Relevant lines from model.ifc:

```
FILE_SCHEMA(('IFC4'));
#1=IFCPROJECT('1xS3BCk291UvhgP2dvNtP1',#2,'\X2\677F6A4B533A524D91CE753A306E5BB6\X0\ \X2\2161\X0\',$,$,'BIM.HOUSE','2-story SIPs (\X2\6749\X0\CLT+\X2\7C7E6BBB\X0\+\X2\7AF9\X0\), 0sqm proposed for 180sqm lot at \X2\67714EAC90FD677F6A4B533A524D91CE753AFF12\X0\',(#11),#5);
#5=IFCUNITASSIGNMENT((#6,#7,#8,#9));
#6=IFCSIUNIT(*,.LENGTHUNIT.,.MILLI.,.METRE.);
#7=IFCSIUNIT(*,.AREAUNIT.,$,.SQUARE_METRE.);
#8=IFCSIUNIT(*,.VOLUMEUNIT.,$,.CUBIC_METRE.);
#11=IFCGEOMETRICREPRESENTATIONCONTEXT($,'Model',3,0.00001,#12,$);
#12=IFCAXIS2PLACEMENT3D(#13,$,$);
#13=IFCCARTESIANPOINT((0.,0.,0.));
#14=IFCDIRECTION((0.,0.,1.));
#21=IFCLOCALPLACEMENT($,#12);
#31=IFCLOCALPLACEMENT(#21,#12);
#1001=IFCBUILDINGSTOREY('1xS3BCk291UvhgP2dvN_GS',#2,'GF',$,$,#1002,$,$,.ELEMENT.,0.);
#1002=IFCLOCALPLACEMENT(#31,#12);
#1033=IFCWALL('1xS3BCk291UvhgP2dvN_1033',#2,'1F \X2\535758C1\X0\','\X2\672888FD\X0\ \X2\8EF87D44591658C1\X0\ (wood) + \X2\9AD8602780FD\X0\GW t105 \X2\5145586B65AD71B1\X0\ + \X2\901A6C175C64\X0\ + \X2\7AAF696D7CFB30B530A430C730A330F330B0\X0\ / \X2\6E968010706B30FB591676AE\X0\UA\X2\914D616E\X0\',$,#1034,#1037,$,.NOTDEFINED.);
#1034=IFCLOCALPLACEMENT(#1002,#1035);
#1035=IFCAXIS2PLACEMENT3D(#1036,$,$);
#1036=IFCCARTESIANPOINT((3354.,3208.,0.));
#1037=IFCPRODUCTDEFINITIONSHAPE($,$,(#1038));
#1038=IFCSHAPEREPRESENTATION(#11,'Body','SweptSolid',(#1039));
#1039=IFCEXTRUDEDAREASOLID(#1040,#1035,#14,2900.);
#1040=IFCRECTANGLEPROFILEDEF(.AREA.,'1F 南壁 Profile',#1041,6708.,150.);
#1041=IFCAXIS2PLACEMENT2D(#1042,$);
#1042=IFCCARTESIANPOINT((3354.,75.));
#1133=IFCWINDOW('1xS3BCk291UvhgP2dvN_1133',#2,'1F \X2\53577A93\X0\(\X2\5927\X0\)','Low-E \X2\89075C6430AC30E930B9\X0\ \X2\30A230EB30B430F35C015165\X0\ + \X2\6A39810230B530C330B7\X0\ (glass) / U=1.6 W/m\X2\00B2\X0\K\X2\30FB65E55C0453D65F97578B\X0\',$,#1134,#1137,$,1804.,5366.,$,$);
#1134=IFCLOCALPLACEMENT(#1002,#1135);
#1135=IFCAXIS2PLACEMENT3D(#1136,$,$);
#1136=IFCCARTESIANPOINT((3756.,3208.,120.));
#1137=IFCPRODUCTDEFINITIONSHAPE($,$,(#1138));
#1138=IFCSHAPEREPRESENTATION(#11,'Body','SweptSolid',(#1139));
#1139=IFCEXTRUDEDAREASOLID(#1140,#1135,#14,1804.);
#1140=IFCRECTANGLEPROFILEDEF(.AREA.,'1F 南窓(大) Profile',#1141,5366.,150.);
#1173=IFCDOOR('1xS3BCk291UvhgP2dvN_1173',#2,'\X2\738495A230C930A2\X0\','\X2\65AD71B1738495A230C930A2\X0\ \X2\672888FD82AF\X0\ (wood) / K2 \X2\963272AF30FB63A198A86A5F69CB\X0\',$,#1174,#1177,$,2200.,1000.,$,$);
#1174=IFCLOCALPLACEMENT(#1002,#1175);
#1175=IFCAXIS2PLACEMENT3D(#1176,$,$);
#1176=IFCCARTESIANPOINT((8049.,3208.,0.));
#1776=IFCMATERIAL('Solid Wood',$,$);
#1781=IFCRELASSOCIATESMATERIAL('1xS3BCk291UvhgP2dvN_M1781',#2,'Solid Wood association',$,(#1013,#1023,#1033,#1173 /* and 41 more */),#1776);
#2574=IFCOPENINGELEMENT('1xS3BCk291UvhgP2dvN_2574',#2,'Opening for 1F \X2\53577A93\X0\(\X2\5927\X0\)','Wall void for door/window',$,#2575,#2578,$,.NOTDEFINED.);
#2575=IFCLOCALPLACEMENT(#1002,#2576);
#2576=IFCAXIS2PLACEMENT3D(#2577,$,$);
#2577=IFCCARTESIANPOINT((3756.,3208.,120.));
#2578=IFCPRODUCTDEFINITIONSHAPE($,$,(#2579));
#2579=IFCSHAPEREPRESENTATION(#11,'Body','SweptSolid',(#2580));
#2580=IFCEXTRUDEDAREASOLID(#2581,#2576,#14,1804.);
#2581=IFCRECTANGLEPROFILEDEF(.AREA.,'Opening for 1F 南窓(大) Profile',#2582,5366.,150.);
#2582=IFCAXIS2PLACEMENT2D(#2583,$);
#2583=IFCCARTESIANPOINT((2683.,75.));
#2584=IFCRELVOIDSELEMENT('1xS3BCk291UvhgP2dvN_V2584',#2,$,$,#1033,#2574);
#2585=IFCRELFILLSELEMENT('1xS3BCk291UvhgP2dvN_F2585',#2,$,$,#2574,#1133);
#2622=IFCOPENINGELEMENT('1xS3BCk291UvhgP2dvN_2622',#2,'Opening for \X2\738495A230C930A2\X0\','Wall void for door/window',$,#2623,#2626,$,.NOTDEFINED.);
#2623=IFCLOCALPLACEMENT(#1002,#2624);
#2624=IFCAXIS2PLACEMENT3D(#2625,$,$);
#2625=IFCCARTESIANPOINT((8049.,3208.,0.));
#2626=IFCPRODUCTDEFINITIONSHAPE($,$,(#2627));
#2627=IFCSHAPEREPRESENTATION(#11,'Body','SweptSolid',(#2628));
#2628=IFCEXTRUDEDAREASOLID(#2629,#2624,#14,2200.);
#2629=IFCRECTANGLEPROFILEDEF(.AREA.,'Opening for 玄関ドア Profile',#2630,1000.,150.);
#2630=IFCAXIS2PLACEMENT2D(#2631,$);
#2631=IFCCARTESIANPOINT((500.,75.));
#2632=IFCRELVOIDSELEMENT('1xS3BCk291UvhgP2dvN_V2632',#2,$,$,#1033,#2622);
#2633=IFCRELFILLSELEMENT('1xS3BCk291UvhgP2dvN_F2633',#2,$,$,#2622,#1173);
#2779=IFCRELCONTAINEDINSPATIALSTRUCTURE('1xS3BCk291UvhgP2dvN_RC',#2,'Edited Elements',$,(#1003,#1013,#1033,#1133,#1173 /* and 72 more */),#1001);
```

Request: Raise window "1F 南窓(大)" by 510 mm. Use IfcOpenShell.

```python
import numpy as np
import ifcopenshell
import ifcopenshell.api.geometry
import ifcopenshell.util.placement
import ifcopenshell.util.unit

model = ifcopenshell.open("model.ifc")
unit_scale = ifcopenshell.util.unit.calculate_unit_scale(model)

window = model.by_id(1133)
opening = window.FillsVoids[0].RelatingOpeningElement
dz = 0.51 / unit_scale

shift = np.array([0.0, 0.0, dz])
# The window is not placed relative to its opening, so move both.
for product in (opening, window):
    matrix = ifcopenshell.util.placement.get_local_placement(product.ObjectPlacement)
    matrix[:3, 3] += shift
    ifcopenshell.api.geometry.edit_object_placement(model, product=product, matrix=matrix, is_si=False)

print(f"moved by {dz * unit_scale:+.3f} m")

model.write("model-out.ifc")
```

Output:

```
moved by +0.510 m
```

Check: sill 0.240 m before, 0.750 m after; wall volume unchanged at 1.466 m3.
